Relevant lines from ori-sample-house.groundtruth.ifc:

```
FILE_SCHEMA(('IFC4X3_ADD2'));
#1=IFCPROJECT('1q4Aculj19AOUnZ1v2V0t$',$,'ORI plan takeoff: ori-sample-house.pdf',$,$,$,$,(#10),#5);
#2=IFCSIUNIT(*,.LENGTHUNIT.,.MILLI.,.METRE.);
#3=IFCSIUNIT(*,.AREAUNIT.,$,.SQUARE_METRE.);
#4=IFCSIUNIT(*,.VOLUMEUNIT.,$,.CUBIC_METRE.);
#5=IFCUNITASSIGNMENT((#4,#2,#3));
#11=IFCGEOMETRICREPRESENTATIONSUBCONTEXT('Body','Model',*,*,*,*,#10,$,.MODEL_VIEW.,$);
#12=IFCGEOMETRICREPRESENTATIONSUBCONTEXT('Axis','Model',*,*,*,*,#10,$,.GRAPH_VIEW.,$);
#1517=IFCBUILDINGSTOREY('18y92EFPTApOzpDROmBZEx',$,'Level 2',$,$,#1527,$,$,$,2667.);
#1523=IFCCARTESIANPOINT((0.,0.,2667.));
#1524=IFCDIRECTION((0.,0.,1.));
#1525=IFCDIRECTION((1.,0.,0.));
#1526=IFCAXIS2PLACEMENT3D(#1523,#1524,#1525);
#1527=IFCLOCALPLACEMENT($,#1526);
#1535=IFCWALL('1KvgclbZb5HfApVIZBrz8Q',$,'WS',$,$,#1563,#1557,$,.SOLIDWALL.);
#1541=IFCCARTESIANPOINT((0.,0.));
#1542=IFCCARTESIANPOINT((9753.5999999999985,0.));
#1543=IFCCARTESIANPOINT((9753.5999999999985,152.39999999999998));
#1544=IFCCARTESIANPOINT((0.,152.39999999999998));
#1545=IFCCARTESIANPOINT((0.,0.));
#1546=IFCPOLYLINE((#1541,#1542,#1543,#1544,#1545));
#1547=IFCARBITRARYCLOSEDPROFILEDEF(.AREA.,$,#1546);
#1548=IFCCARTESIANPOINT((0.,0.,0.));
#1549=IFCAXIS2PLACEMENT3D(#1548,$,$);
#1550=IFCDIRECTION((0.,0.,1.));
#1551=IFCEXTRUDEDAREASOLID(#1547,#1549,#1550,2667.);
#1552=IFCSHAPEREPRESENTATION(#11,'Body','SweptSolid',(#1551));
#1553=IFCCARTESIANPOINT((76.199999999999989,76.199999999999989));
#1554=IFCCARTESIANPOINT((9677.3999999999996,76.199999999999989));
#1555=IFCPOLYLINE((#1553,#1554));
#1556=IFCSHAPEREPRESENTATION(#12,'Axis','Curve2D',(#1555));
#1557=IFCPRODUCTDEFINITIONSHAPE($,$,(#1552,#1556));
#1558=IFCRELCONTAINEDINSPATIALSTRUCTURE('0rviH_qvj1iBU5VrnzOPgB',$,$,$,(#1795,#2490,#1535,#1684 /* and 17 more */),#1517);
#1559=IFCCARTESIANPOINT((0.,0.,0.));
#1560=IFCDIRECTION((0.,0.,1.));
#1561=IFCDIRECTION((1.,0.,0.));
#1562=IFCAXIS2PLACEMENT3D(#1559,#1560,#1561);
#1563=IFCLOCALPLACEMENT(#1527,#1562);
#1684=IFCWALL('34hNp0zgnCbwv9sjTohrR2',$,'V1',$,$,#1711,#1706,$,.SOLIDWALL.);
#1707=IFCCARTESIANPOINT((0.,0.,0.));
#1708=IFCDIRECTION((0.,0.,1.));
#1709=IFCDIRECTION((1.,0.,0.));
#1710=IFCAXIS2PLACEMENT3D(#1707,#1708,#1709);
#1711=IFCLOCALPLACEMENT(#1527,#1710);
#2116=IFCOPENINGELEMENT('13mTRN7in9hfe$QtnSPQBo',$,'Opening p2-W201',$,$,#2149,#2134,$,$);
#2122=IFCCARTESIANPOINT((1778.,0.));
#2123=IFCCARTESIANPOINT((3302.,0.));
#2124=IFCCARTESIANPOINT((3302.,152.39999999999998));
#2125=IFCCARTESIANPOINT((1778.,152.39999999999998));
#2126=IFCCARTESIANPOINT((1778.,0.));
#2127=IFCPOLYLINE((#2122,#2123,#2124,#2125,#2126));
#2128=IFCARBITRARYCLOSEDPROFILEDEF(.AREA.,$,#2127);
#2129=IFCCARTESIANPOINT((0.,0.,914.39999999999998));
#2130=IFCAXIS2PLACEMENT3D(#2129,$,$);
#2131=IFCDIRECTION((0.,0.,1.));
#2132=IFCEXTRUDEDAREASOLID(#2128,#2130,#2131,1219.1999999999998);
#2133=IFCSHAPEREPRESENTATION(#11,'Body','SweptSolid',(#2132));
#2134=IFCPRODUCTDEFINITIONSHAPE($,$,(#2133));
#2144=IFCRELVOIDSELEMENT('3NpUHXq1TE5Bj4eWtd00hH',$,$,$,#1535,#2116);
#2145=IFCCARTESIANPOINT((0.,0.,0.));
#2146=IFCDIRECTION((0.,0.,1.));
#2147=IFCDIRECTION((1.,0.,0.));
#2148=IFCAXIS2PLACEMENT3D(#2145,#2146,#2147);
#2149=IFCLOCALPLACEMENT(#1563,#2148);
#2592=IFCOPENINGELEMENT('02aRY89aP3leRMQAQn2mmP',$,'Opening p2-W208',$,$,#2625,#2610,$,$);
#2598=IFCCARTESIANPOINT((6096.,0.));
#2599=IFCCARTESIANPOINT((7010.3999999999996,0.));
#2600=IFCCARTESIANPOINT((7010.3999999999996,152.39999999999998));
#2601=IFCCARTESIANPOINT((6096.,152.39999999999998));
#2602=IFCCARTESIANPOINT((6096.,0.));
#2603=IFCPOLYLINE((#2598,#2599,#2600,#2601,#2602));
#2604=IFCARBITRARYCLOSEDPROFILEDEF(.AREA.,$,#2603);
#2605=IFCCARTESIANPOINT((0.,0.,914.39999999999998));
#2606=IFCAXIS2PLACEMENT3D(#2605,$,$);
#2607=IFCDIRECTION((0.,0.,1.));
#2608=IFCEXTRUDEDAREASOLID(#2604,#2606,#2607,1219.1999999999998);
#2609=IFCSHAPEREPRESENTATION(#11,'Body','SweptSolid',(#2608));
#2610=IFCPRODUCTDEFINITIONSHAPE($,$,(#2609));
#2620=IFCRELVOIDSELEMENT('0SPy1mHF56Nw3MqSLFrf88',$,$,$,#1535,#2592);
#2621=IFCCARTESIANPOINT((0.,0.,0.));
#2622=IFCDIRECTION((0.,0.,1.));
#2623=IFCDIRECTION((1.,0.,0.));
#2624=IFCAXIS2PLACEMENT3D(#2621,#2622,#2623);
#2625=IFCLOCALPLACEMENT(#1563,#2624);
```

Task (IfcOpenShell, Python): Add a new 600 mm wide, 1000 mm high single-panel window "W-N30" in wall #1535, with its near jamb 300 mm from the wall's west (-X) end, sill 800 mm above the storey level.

```python
import numpy as np
import ifcopenshell
import ifcopenshell.api.feature
import ifcopenshell.api.geometry
import ifcopenshell.api.root
import ifcopenshell.api.spatial
import ifcopenshell.geom
import ifcopenshell.util.element
import ifcopenshell.util.placement
import ifcopenshell.util.representation
import ifcopenshell.util.shape
import ifcopenshell.util.unit

model = ifcopenshell.open("ori-sample-house.groundtruth.ifc")
unit_scale = ifcopenshell.util.unit.calculate_unit_scale(model)
settings = ifcopenshell.geom.settings()


def volume(element):
    """Net volume in cubic metres, openings subtracted."""
    shape = ifcopenshell.geom.create_shape(settings, element)
    return ifcopenshell.util.shape.get_volume(shape.geometry)


wall = model.by_id(1535)
storey = ifcopenshell.util.element.get_container(wall, ifc_class="IfcBuildingStorey")
context = ifcopenshell.util.representation.get_context(model, "Model", "Body", "MODEL_VIEW")
before = volume(wall)

width, height, from_end, sill = 0.6, 1, 0.3, 0.8  # metres

# The wall runs along its own X axis, and the end named is its -X end.
wall_shape = ifcopenshell.geom.create_shape(settings, wall)
x, y, z = ifcopenshell.util.shape.get_vertices(wall_shape.geometry).T
start = x.min() + from_end
face, thickness = float(y.min()), float(y.max() - y.min())
wall_matrix = ifcopenshell.util.placement.get_local_placement(wall.ObjectPlacement)
level = ifcopenshell.util.placement.get_local_placement(storey.ObjectPlacement)[2, 3]


def in_wall(x, y):
    """Placement at x, y metres in the wall's axes, at sill height."""
    matrix = wall_matrix.copy()
    matrix[:, 3] = wall_matrix @ np.array([x / unit_scale, y / unit_scale, 0.0, 1.0])
    matrix[2, 3] = level + sill / unit_scale
    return matrix


# Opening: a box that overshoots both wall faces by 50 mm.
opening = ifcopenshell.api.root.create_entity(model, ifc_class="IfcOpeningElement", predefined_type="OPENING")
box = ifcopenshell.api.geometry.add_wall_representation(
    model, context=context, length=width, height=height, thickness=thickness + 0.1
)
ifcopenshell.api.geometry.assign_representation(model, product=opening, representation=box)
ifcopenshell.api.geometry.edit_object_placement(model, product=opening, matrix=in_wall(start, face - 0.05), is_si=False)
ifcopenshell.api.feature.add_feature(model, feature=opening, element=wall)

window = ifcopenshell.api.root.create_entity(model, ifc_class="IfcWindow", name="W-N30", predefined_type="WINDOW")
window.OverallWidth, window.OverallHeight = width / unit_scale, height / unit_scale
window.PartitioningType = "SINGLE_PANEL"
body = ifcopenshell.api.geometry.add_window_representation(
    model,
    context=context,
    overall_width=window.OverallWidth,
    overall_height=window.OverallHeight,
    partition_type="SINGLE_PANEL",
)
ifcopenshell.api.geometry.assign_representation(model, product=window, representation=body)
ifcopenshell.api.spatial.assign_container(model, products=[window], relating_structure=storey)
ifcopenshell.api.feature.add_filling(model, opening=opening, element=window)

# Centre the window in the wall's thickness.
ifcopenshell.api.geometry.edit_object_placement(model, product=window, matrix=in_wall(start, face), is_si=False)
window_shape = ifcopenshell.geom.create_shape(settings, window)
depth = ifcopenshell.util.shape.get_vertices(window_shape.geometry)[:, 1]
offset = face + thickness / 2 - (depth.min() + depth.max()) / 2
ifcopenshell.api.geometry.edit_object_placement(model, product=window, matrix=in_wall(start, offset), is_si=False)

after = volume(wall)

print(f"wall volume {before:.3f} -> {after:.3f} m3")

model.write("ori-sample-house.groundtruth_rev.ifc")
```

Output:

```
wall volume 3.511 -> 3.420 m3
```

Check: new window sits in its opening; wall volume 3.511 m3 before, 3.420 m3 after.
